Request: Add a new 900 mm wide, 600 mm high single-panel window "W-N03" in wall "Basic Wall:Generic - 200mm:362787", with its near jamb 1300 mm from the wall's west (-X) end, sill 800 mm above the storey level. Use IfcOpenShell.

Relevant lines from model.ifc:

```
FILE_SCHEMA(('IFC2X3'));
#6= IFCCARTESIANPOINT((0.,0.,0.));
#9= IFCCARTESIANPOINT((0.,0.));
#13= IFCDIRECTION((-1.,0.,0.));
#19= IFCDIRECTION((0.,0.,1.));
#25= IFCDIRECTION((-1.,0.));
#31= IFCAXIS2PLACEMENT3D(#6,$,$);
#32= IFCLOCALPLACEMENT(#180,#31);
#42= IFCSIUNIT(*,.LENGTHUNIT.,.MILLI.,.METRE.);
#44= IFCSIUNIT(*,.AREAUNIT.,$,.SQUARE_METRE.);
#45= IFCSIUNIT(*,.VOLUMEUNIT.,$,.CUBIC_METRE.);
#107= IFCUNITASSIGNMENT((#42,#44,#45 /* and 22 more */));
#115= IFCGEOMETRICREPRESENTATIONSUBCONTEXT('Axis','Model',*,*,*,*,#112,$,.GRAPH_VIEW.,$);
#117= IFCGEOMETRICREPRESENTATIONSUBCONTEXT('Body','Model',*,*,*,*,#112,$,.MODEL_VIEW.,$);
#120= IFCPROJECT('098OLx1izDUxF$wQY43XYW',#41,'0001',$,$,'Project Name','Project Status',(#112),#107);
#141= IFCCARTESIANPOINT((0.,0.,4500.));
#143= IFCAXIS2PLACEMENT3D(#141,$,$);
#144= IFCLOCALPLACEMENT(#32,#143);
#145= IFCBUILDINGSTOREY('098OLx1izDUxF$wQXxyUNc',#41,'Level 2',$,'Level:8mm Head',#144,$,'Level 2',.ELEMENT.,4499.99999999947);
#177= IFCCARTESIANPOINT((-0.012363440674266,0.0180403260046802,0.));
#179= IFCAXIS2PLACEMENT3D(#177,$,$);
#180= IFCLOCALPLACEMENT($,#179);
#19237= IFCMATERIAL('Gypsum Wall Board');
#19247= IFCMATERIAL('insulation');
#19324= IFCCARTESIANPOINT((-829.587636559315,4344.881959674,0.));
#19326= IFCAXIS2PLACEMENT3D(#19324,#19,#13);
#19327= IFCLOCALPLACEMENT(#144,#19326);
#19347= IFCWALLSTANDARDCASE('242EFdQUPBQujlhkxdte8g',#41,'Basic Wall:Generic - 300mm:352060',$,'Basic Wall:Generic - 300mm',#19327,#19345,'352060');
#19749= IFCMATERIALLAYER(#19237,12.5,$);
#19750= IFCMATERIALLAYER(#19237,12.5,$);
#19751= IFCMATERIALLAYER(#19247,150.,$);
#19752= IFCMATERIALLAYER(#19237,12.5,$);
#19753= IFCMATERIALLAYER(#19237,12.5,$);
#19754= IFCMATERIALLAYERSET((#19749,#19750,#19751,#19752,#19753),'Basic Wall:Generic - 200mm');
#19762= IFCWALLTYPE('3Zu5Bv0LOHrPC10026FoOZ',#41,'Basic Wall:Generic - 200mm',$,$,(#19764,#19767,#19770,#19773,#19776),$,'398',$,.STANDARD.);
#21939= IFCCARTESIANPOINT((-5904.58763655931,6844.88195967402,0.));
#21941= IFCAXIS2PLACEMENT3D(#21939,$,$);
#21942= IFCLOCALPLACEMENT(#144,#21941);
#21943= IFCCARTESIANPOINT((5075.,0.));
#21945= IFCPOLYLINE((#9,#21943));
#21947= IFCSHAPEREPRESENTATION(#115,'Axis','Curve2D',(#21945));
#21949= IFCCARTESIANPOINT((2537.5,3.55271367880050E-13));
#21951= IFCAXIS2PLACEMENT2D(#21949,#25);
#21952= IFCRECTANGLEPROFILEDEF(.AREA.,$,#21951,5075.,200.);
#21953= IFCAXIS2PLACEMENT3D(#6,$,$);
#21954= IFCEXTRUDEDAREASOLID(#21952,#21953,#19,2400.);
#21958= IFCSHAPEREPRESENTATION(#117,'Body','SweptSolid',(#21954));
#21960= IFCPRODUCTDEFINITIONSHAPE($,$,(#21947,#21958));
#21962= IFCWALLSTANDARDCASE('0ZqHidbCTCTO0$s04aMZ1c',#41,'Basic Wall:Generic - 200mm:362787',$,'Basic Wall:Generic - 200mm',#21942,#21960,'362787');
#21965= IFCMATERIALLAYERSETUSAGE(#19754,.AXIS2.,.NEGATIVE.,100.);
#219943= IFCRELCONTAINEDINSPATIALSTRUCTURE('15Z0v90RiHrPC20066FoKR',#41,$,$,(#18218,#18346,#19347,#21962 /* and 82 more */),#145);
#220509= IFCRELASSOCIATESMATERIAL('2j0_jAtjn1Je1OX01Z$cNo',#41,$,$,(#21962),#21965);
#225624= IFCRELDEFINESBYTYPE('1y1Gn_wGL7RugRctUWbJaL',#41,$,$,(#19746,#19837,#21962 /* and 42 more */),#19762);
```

```python
import numpy as np
import ifcopenshell
import ifcopenshell.api.feature
import ifcopenshell.api.geometry
import ifcopenshell.api.root
import ifcopenshell.api.spatial
import ifcopenshell.api.type
import ifcopenshell.geom
import ifcopenshell.util.element
import ifcopenshell.util.placement
import ifcopenshell.util.representation
import ifcopenshell.util.shape
import ifcopenshell.util.unit

model = ifcopenshell.open("model.ifc")
unit_scale = ifcopenshell.util.unit.calculate_unit_scale(model)
settings = ifcopenshell.geom.settings()


def volume(element):
    """Net volume in cubic metres, openings subtracted."""
    shape = ifcopenshell.geom.create_shape(settings, element)
    return ifcopenshell.util.shape.get_volume(shape.geometry)


wall = model.by_guid("0ZqHidbCTCTO0$s04aMZ1c")
storey = ifcopenshell.util.element.get_container(wall, ifc_class="IfcBuildingStorey")
context = ifcopenshell.util.representation.get_context(model, "Model", "Body", "MODEL_VIEW")
before = volume(wall)

width, height, from_end, sill = 0.9, 0.6, 1.3, 0.8  # metres

# The wall runs along its own X axis, and the end named is its -X end.
wall_shape = ifcopenshell.geom.create_shape(settings, wall)
x, y, z = ifcopenshell.util.shape.get_vertices(wall_shape.geometry).T
start = x.min() + from_end
face, thickness = float(y.min()), float(y.max() - y.min())
wall_matrix = ifcopenshell.util.placement.get_local_placement(wall.ObjectPlacement)
level = ifcopenshell.util.placement.get_local_placement(storey.ObjectPlacement)[2, 3]


def in_wall(x, y):
    """Placement at x, y metres in the wall's axes, at sill height."""
    matrix = wall_matrix.copy()
    matrix[:, 3] = wall_matrix @ np.array([x / unit_scale, y / unit_scale, 0.0, 1.0])
    matrix[2, 3] = level + sill / unit_scale
    return matrix


# Opening: a box that overshoots both wall faces by 50 mm.
opening = ifcopenshell.api.root.create_entity(model, ifc_class="IfcOpeningElement")
box = ifcopenshell.api.geometry.add_wall_representation(
    model, context=context, length=width, height=height, thickness=thickness + 0.1
)
ifcopenshell.api.geometry.assign_representation(model, product=opening, representation=box)
ifcopenshell.api.geometry.edit_object_placement(model, product=opening, matrix=in_wall(start, face - 0.05), is_si=False)
ifcopenshell.api.feature.add_feature(model, feature=opening, element=wall)

window = ifcopenshell.api.root.create_entity(model, ifc_class="IfcWindow", name="W-N03")
window.OverallWidth, window.OverallHeight = width / unit_scale, height / unit_scale
body = ifcopenshell.api.geometry.add_window_representation(
    model,
    context=context,
    overall_width=window.OverallWidth,
    overall_height=window.OverallHeight,
    partition_type="SINGLE_PANEL",
)
ifcopenshell.api.geometry.assign_representation(model, product=window, representation=body)
ifcopenshell.api.spatial.assign_container(model, products=[window], relating_structure=storey)
fills = ifcopenshell.api.feature.add_filling(model, opening=opening, element=window)
fills.OwnerHistory = window.OwnerHistory  # required in IFC2X3

# IFC2X3 keeps the operation on the window style.
style = ifcopenshell.api.root.create_entity(model, ifc_class="IfcWindowStyle", name="W-N03")
style.OperationType, style.ConstructionType = "SINGLE_PANEL", "NOTDEFINED"
style.ParameterTakesPrecedence = style.Sizeable = False
ifcopenshell.api.type.assign_type(model, related_objects=[window], relating_type=style)

# Centre the window in the wall's thickness.
ifcopenshell.api.geometry.edit_object_placement(model, product=window, matrix=in_wall(start, face), is_si=False)
window_shape = ifcopenshell.geom.create_shape(settings, window)
depth = ifcopenshell.util.shape.get_vertices(window_shape.geometry)[:, 1]
offset = face + thickness / 2 - (depth.min() + depth.max()) / 2
ifcopenshell.api.geometry.edit_object_placement(model, product=window, matrix=in_wall(start, offset), is_si=False)

after = volume(wall)

print(f"wall volume {before:.3f} -> {after:.3f} m3")

model.write("model_rev.ifc")
```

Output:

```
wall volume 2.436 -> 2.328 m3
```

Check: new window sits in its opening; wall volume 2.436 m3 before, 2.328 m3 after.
